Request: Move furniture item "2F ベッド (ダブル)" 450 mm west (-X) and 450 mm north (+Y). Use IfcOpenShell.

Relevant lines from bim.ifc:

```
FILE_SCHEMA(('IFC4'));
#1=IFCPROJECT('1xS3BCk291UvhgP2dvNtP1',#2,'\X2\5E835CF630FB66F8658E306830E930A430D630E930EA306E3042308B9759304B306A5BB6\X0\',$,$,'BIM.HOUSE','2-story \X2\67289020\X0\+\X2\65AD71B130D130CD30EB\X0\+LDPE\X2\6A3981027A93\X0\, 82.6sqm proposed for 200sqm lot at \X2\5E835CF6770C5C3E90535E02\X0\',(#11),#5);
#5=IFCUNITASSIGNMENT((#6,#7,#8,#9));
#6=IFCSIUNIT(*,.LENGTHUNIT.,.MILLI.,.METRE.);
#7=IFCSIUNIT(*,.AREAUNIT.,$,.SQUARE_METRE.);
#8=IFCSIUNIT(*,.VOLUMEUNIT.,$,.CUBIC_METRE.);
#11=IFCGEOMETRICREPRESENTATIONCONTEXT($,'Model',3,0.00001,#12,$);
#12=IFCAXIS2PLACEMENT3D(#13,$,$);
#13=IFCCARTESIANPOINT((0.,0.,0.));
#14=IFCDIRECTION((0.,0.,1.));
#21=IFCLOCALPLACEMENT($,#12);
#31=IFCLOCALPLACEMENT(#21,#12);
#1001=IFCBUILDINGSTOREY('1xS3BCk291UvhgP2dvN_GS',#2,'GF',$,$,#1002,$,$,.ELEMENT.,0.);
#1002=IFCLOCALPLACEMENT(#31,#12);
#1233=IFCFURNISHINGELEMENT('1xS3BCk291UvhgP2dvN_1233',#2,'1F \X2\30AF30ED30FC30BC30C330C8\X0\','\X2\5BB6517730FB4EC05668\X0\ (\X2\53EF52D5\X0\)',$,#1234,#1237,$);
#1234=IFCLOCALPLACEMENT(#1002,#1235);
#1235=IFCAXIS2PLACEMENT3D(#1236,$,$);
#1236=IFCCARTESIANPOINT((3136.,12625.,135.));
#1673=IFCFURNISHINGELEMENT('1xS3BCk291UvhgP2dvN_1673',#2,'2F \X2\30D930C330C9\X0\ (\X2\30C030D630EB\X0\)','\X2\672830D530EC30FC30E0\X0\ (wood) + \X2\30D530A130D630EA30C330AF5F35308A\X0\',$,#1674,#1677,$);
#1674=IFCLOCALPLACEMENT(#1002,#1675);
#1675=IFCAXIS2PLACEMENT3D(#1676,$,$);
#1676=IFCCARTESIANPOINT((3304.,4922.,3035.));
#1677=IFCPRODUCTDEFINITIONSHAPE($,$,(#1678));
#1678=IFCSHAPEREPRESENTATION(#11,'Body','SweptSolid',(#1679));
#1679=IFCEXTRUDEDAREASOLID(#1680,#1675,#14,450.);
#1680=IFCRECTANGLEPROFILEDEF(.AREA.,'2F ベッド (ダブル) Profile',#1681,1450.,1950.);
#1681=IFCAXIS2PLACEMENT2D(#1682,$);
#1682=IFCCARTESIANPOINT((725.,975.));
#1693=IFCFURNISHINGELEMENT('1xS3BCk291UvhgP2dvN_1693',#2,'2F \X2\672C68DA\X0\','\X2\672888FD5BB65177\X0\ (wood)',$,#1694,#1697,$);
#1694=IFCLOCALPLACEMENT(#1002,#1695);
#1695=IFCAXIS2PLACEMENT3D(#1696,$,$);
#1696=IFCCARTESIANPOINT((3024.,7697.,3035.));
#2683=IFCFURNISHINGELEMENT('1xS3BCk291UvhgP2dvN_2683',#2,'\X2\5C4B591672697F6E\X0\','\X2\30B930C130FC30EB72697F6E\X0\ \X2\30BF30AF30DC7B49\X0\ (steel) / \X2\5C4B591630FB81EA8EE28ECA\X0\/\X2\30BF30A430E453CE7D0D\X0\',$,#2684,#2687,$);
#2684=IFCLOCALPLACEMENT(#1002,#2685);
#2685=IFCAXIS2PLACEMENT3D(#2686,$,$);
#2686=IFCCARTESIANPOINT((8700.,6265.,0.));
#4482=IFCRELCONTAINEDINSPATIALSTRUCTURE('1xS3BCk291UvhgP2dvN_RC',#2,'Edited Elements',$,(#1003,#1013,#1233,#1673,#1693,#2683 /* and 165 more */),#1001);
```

```python
import ifcopenshell
import ifcopenshell.api.geometry
import ifcopenshell.util.placement
import ifcopenshell.util.unit

model = ifcopenshell.open("bim.ifc")
unit_scale = ifcopenshell.util.unit.calculate_unit_scale(model)

item = model.by_id(1673)
matrix = ifcopenshell.util.placement.get_local_placement(item.ObjectPlacement)
matrix[0, 3] -= 0.45 / unit_scale
matrix[1, 3] += 0.45 / unit_scale
ifcopenshell.api.geometry.edit_object_placement(model, product=item, matrix=matrix, is_si=False)

print(ifcopenshell.util.placement.get_local_placement(item.ObjectPlacement).round(3) + 0.0)

model.write("bim_updated.ifc")
```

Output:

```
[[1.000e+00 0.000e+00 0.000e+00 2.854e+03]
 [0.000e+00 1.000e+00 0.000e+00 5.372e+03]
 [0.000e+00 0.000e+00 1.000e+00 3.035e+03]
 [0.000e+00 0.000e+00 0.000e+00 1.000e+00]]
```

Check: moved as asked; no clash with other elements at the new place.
